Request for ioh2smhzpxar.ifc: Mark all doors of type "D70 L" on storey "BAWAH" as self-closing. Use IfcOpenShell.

First a look at what the model holds.

```python
import ifcopenshell
import ifcopenshell.util.element

model = ifcopenshell.open("ioh2smhzpxar.ifc")
print(model.schema)
storey = next(s for s in model.by_type("IfcBuildingStorey") if s.Name == "BAWAH")
doors = [e for e in ifcopenshell.util.element.get_decomposition(storey) if e.is_a("IfcDoor")]
seen = {}
for e in doors:
    element_type = ifcopenshell.util.element.get_type(e)
    key = (element_type.Name if element_type != e and element_type else None, ifcopenshell.util.element.get_pset(e, "Pset_DoorCommon", "SelfClosing"))
    seen[key] = seen.get(key, 0) + 1
for (name, value), count in sorted(seen.items(), key=str):
    print(count, "x", name, "|", value)
```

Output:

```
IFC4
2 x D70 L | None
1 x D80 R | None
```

```python
import ifcopenshell
import ifcopenshell.api.pset
import ifcopenshell.util.element

model = ifcopenshell.open("ioh2smhzpxar.ifc")

storey = next(s for s in model.by_type("IfcBuildingStorey") if s.Name == "BAWAH")
doors = [e for e in ifcopenshell.util.element.get_decomposition(storey) if e.is_a("IfcDoor")]

count = 0
for e in doors:
    element_type = ifcopenshell.util.element.get_type(e)
    if element_type in (None, e) or element_type.Name != "D70 L":
        continue
    # add_pset returns the element's existing set when there is one.
    pset = ifcopenshell.api.pset.add_pset(model, product=e, name="Pset_DoorCommon")
    ifcopenshell.api.pset.edit_pset(model, pset=pset, properties={"SelfClosing": True})
    count += 1

print(count, "doors updated")

model.write("ioh2smhzpxar_v2.ifc")
```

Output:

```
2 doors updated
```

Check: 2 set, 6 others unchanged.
